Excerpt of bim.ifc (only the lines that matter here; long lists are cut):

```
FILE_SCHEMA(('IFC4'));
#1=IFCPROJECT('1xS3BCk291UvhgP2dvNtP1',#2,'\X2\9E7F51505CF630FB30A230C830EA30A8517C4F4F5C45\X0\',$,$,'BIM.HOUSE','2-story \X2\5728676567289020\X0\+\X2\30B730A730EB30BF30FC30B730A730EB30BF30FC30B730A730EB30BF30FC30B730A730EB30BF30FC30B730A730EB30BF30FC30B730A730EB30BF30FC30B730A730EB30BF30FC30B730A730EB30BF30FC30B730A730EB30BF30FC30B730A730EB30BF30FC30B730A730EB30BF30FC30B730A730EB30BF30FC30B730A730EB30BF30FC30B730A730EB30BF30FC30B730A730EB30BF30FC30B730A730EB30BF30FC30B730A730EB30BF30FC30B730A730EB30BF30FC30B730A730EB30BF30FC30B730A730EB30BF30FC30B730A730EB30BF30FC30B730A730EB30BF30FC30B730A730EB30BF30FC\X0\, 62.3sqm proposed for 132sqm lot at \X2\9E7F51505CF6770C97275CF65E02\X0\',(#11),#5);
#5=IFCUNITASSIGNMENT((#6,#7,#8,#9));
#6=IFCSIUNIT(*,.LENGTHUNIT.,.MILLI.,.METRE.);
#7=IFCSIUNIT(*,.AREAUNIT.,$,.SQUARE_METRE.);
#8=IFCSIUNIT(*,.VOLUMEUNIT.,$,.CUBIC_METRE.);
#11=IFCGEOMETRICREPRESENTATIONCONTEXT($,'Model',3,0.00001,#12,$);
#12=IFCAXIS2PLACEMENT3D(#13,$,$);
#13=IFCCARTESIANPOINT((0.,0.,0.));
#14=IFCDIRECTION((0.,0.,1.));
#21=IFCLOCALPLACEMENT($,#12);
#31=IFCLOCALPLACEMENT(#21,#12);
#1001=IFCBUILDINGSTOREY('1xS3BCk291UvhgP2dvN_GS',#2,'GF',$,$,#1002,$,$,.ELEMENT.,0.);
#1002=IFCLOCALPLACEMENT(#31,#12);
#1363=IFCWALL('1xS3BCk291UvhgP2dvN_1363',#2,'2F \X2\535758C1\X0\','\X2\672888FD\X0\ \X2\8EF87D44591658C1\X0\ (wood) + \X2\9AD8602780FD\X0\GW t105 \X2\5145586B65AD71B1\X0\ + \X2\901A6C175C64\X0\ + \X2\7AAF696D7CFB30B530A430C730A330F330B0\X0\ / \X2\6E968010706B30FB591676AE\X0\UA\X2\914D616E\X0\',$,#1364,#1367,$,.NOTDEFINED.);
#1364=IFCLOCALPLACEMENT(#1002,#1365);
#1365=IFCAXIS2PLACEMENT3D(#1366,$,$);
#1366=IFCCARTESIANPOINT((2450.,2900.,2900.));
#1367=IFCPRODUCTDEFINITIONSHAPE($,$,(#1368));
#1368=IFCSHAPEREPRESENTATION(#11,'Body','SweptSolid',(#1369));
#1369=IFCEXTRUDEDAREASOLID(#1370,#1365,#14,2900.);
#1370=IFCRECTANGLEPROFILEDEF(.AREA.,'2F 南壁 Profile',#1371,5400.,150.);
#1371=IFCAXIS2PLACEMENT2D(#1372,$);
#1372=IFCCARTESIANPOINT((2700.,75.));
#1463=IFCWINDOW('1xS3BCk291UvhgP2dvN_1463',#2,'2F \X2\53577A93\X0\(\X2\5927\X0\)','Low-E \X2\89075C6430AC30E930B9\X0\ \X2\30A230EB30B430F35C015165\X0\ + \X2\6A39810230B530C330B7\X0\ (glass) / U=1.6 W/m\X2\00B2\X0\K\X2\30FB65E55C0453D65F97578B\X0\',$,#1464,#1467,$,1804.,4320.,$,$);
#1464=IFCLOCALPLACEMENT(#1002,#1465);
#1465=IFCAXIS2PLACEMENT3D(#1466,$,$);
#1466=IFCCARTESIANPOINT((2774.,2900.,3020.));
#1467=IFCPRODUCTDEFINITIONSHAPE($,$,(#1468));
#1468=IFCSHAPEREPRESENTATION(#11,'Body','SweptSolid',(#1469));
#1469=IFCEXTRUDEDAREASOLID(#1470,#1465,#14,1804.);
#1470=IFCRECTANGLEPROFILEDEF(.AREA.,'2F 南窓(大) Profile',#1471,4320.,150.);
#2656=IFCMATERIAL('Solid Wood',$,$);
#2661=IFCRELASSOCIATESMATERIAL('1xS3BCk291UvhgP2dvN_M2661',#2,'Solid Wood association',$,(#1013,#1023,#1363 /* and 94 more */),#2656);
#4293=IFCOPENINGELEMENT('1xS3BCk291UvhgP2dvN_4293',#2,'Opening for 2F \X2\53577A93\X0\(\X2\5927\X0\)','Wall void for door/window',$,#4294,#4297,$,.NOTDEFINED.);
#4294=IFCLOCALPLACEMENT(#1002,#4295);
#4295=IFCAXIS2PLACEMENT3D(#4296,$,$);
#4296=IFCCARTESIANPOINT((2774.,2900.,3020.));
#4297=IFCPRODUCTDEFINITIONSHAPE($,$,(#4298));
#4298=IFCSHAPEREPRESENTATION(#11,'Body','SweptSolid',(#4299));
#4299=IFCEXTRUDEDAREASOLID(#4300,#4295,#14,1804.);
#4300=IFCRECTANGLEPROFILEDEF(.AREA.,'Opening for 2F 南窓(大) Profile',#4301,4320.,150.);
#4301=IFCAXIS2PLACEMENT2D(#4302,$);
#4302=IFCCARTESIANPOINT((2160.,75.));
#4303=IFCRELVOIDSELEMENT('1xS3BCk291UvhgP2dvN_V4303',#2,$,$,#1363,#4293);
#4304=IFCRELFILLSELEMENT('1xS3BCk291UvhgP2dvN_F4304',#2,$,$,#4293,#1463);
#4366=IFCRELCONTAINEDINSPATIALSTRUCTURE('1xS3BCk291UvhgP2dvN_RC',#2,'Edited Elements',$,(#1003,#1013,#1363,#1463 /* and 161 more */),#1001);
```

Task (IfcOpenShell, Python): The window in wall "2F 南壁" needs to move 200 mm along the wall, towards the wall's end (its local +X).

```python
import ifcopenshell
import ifcopenshell.api.geometry
import ifcopenshell.util.placement

model = ifcopenshell.open("bim.ifc")

window = model.by_guid("1xS3BCk291UvhgP2dvN_1463")
opening = window.FillsVoids[0].RelatingOpeningElement
wall = opening.VoidsElements[0].RelatingBuildingElement

wall_matrix = ifcopenshell.util.placement.get_local_placement(wall.ObjectPlacement)
shift = wall_matrix[:3, 0] * 200.0
before = ifcopenshell.util.placement.get_local_placement(window.ObjectPlacement)[:3, 3].copy()

# The window is not placed relative to its opening, so move both.
for product in (opening, window):
    matrix = ifcopenshell.util.placement.get_local_placement(product.ObjectPlacement)
    matrix[:3, 3] += shift
    ifcopenshell.api.geometry.edit_object_placement(model, product=product, matrix=matrix, is_si=False)

after = ifcopenshell.util.placement.get_local_placement(window.ObjectPlacement)[:3, 3]
print("window moved by", (after - before).round(3) + 0.0)

model.write("bim_v2.ifc")
```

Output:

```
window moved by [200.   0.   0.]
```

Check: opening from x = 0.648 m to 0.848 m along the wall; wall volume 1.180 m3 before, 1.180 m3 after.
